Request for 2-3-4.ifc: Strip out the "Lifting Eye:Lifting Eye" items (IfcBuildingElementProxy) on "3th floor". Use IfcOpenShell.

First a look at what the model holds.

```python
import ifcopenshell
import ifcopenshell.util.element

model = ifcopenshell.open("2-3-4.ifc")
print(model.schema)
storey = next(s for s in model.by_type("IfcBuildingStorey") if s.Name == "3th floor")
proxies = [e for e in ifcopenshell.util.element.get_decomposition(storey) if e.is_a("IfcBuildingElementProxy")]
seen = {}
for e in proxies:
    element_type = ifcopenshell.util.element.get_type(e)
    name = element_type.Name if element_type not in (None, e) else None
    seen[name] = seen.get(name, 0) + 1
for name, count in sorted(seen.items(), key=str):
    print(count, "x", name)
```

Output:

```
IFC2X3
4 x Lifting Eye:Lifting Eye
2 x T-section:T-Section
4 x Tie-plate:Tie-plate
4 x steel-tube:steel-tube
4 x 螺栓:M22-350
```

```python
import ifcopenshell
import ifcopenshell.api.root
import ifcopenshell.util.element

model = ifcopenshell.open("2-3-4.ifc")

storey = next(s for s in model.by_type("IfcBuildingStorey") if s.Name == "3th floor")
proxies = [e for e in ifcopenshell.util.element.get_decomposition(storey) if e.is_a("IfcBuildingElementProxy")]
targets = [e for e in proxies if (t := ifcopenshell.util.element.get_type(e)) not in (None, e) and t.Name == "Lifting Eye:Lifting Eye"]

for e in targets:
    ifcopenshell.api.root.remove_product(model, product=e)
print(len(targets), "removed")

model.write("2-3-4_updated.ifc")
```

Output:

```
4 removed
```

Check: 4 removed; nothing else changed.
